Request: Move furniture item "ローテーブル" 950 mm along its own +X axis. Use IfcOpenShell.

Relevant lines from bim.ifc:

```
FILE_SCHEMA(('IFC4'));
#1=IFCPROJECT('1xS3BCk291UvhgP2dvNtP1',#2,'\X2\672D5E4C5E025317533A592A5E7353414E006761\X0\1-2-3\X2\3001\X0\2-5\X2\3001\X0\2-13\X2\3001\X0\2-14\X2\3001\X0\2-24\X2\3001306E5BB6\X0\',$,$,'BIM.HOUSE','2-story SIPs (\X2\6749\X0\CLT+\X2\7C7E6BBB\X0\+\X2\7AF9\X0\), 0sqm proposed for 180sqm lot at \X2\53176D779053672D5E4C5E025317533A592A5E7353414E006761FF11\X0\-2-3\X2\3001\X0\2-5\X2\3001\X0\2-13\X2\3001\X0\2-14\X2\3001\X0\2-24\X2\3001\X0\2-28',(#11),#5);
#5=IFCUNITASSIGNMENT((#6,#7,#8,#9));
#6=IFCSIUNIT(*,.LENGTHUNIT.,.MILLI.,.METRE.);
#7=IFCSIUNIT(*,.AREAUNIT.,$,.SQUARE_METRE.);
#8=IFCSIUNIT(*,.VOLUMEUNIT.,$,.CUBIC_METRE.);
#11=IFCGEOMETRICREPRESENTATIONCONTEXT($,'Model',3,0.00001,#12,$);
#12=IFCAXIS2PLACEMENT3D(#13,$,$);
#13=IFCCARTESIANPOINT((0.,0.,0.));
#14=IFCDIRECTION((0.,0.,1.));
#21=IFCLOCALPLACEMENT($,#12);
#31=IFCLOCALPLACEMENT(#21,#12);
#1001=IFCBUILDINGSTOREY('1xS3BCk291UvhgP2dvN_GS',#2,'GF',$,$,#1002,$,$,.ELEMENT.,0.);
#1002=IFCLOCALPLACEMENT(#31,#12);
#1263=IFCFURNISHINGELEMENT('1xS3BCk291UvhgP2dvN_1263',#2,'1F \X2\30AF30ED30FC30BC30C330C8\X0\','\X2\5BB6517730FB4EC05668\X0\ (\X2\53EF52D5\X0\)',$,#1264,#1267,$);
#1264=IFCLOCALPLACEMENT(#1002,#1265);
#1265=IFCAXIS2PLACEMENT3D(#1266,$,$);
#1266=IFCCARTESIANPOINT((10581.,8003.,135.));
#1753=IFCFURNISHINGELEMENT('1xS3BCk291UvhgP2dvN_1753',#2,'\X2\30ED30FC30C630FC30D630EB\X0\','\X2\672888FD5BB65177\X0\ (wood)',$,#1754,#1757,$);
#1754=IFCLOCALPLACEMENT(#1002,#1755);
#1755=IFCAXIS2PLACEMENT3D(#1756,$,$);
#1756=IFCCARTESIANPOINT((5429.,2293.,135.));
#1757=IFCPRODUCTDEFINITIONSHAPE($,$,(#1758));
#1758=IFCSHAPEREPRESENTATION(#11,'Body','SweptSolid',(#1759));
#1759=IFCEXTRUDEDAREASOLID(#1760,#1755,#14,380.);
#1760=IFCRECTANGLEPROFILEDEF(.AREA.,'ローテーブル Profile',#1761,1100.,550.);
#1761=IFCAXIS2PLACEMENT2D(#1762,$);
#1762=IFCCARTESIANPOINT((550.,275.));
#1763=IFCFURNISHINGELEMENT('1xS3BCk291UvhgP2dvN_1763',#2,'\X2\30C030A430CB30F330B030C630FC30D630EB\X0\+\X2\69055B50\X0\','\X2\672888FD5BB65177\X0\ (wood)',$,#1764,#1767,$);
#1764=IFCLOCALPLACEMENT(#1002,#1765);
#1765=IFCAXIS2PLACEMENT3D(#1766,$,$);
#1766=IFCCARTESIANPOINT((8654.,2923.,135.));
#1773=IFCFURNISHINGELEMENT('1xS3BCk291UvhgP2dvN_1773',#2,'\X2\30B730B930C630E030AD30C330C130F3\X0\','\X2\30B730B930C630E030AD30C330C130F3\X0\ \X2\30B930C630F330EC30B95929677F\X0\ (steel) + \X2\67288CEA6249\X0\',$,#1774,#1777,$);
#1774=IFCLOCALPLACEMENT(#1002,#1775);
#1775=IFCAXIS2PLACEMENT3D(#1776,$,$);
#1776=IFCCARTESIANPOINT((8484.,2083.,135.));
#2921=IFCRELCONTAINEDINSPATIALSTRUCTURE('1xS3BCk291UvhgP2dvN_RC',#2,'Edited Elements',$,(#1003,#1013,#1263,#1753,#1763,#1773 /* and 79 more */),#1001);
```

```python
import ifcopenshell
import ifcopenshell.api.geometry
import ifcopenshell.util.placement
import ifcopenshell.util.unit

model = ifcopenshell.open("bim.ifc")
unit_scale = ifcopenshell.util.unit.calculate_unit_scale(model)

item = model.by_guid("1xS3BCk291UvhgP2dvN_1753")
matrix = ifcopenshell.util.placement.get_local_placement(item.ObjectPlacement)
matrix[:3, 3] += matrix[:3, 0] * 0.95 / unit_scale
ifcopenshell.api.geometry.edit_object_placement(model, product=item, matrix=matrix, is_si=False)

print(ifcopenshell.util.placement.get_local_placement(item.ObjectPlacement).round(3) + 0.0)

model.write("bim_updated.ifc")
```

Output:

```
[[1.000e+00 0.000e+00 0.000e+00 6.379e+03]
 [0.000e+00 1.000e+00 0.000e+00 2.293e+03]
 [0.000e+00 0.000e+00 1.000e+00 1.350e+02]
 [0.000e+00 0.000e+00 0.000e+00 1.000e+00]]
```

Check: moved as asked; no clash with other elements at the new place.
